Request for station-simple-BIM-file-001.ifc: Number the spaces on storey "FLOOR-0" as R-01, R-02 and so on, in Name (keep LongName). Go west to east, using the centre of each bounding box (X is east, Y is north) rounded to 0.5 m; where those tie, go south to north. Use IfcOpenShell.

First a look at what the model holds.

```python
import ifcopenshell
import ifcopenshell.util.element
import ifcopenshell.util.placement

model = ifcopenshell.open("station-simple-BIM-file-001.ifc")
print(model.schema)
storey = next(s for s in model.by_type("IfcBuildingStorey") if s.Name == "FLOOR-0")
spaces = [e for e in ifcopenshell.util.element.get_decomposition(storey) if e.is_a("IfcSpace")]
for e in sorted(spaces, key=lambda e: e.id()):
    origin = ifcopenshell.util.placement.get_local_placement(e.ObjectPlacement)[:3, 3]
    print(e.id(), e.Name, e.LongName, origin.round(2) + 0.0, sep=" | ")
```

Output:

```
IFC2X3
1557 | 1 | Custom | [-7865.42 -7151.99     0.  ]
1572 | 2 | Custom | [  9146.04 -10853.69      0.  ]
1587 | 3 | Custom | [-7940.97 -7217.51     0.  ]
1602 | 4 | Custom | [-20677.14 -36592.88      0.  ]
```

```python
import ifcopenshell
import ifcopenshell.geom
import ifcopenshell.util.element
import ifcopenshell.util.shape

model = ifcopenshell.open("station-simple-BIM-file-001.ifc")
settings = ifcopenshell.geom.settings()
settings.set("use-world-coords", True)


def centre(element):
    shape = ifcopenshell.geom.create_shape(settings, element)
    return ifcopenshell.util.shape.get_bbox_centroid(shape.geometry)


storey = next(s for s in model.by_type("IfcBuildingStorey") if s.Name == "FLOOR-0")
spaces = [e for e in ifcopenshell.util.element.get_decomposition(storey) if e.is_a("IfcSpace")]

# Insertion points can sit at a corner or the storey origin, so sort by the geometry (in metres).
centres = {e: centre(e) for e in spaces}
spaces.sort(key=lambda e: (round(centres[e][0] / 0.5), centres[e][1]))

for i, e in enumerate(spaces, start=1):
    number = f"R-{i:02d}"
    e.Name = number
    print(e.id(), number)

model.write("station-simple-BIM-file-001-out.ifc")
```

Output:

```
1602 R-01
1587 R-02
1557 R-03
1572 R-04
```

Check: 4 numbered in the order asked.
